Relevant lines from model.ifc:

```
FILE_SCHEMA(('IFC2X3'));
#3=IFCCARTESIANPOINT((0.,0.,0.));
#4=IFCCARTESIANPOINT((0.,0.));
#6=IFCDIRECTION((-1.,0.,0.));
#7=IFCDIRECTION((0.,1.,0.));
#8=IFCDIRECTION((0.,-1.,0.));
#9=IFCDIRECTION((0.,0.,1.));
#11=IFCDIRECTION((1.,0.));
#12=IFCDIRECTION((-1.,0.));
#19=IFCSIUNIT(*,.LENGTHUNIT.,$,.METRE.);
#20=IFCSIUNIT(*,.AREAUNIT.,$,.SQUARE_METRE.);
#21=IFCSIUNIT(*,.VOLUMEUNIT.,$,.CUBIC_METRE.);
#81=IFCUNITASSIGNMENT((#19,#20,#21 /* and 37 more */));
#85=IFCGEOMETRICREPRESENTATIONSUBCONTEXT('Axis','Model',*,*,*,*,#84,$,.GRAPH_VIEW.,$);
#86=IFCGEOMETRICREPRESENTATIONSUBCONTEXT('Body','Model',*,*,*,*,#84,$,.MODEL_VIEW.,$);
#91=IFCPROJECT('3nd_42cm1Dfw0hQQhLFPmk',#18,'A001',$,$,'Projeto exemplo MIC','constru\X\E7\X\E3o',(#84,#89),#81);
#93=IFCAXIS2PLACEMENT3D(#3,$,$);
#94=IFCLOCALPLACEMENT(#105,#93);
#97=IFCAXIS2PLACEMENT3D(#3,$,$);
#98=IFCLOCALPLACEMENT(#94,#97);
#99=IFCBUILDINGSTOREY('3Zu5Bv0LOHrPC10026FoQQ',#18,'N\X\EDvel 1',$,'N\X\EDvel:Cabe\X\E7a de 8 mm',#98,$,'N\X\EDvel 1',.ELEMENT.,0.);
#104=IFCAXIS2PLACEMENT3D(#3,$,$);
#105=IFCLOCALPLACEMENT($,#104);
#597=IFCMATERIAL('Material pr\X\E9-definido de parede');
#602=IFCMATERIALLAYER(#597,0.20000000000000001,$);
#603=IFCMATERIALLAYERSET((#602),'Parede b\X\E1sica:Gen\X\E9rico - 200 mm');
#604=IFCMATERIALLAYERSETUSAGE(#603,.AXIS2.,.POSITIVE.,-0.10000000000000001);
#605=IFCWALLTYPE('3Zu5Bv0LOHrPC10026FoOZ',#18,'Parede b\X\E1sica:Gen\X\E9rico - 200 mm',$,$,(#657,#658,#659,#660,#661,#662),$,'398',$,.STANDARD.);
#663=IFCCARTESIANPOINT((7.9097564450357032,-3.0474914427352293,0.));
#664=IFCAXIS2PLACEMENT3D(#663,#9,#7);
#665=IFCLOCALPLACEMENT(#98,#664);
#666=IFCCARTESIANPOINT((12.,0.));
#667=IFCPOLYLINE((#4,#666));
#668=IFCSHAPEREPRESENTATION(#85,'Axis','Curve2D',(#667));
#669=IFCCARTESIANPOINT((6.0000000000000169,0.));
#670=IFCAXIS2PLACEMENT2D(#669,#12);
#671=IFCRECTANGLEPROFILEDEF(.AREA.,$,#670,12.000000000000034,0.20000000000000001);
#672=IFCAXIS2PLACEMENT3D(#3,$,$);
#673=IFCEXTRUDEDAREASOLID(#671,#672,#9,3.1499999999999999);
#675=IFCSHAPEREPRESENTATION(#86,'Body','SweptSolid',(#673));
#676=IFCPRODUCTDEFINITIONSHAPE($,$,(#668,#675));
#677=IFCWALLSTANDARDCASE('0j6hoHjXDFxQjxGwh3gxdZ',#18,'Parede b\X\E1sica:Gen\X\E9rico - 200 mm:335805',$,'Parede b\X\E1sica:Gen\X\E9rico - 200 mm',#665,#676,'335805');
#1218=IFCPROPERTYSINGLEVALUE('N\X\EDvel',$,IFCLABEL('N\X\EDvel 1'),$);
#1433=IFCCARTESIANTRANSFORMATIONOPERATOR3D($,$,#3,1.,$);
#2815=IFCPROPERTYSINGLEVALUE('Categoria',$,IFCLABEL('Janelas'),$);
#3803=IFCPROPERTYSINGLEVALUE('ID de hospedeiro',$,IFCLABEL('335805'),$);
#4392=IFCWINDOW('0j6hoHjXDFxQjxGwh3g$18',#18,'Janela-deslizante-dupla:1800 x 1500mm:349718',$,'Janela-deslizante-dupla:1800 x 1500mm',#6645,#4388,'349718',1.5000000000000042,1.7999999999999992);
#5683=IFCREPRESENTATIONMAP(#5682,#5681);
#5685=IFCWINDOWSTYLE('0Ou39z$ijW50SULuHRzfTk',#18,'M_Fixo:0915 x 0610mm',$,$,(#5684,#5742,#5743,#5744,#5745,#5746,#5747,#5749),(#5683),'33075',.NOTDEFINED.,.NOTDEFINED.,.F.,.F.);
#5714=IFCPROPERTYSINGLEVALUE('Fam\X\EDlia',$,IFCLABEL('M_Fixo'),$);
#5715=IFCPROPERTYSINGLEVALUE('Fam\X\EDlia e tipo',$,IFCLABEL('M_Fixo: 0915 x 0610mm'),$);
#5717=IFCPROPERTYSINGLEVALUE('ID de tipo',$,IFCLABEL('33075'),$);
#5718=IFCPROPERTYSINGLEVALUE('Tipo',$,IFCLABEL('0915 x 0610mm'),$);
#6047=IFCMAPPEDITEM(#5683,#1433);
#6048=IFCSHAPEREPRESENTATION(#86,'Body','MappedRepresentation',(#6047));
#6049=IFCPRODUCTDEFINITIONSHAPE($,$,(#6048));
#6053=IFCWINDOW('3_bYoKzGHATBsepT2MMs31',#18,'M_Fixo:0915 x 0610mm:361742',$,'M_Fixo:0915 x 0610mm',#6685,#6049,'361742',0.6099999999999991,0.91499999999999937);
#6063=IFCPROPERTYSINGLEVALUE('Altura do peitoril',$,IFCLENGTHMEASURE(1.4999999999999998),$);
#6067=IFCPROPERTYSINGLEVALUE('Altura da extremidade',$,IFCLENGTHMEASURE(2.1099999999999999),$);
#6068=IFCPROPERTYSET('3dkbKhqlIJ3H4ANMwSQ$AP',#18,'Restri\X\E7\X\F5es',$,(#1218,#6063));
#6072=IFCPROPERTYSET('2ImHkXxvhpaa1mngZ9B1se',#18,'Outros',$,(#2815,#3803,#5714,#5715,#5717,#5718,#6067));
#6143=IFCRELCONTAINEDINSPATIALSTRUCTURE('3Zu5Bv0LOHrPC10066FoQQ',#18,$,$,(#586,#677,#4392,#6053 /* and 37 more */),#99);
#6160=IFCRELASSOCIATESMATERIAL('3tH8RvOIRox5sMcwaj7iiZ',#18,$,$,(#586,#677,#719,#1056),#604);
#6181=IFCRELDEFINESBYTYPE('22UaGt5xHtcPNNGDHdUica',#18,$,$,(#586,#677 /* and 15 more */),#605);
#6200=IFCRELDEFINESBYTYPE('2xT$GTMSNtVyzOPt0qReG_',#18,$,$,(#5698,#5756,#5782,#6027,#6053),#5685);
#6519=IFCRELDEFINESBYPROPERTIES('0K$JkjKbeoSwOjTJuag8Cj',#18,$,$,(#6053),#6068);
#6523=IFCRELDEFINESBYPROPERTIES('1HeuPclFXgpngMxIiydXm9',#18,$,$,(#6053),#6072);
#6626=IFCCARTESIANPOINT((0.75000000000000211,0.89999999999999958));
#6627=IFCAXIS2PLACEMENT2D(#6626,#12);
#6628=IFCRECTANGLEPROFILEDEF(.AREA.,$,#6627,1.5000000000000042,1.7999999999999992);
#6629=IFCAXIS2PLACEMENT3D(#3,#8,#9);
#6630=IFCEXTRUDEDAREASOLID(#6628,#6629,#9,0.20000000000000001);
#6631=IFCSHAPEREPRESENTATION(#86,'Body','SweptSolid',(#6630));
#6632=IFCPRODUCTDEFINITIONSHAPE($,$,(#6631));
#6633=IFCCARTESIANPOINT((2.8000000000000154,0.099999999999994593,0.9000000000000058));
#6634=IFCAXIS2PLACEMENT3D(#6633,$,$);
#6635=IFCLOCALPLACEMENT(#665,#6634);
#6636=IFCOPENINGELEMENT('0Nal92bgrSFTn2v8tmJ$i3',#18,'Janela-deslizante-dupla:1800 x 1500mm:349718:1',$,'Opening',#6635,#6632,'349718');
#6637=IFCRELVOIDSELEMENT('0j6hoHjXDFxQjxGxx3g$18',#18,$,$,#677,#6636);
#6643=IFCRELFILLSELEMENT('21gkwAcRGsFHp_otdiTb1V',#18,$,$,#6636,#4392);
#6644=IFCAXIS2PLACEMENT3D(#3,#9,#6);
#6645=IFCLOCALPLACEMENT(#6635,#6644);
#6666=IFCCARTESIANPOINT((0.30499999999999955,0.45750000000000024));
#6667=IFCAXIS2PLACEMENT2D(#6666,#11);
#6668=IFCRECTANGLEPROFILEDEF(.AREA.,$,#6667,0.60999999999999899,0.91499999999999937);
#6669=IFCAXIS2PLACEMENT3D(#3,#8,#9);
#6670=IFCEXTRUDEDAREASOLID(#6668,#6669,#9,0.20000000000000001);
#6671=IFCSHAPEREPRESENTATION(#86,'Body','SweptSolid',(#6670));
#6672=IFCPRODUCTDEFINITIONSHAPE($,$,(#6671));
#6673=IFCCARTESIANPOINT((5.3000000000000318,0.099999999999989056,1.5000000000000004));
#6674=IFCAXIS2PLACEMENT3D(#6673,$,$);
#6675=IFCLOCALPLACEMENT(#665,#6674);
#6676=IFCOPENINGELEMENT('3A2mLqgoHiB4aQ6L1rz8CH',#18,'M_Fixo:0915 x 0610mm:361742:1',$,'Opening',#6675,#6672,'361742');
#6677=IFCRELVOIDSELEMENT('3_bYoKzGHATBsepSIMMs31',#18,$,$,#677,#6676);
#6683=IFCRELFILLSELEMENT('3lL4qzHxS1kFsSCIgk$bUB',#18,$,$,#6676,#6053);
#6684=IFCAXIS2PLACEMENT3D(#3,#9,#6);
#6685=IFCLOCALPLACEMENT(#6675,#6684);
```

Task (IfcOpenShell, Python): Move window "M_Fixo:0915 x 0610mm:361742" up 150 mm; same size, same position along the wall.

```python
import numpy as np
import ifcopenshell
import ifcopenshell.api.geometry
import ifcopenshell.api.pset
import ifcopenshell.util.element
import ifcopenshell.util.placement
import ifcopenshell.util.unit

model = ifcopenshell.open("model.ifc")
unit_scale = ifcopenshell.util.unit.calculate_unit_scale(model)

window = model.by_guid("3_bYoKzGHATBsepT2MMs31")
opening = window.FillsVoids[0].RelatingOpeningElement
dz = 0.15

shift = np.array([0.0, 0.0, dz])
# The window is placed relative to its opening, so it follows when the opening moves.
matrix = ifcopenshell.util.placement.get_local_placement(opening.ObjectPlacement)
matrix[:3, 3] += shift
ifcopenshell.api.geometry.edit_object_placement(
    model, product=opening, matrix=matrix, is_si=False, should_transform_children=True
)

# Keep the stored heights in step.
pset = model.by_id(ifcopenshell.util.element.get_pset(window, "Restrições", should_inherit=False)["id"])
ifcopenshell.api.pset.edit_pset(model, pset=pset, properties={
    "Altura do peitoril": model.create_entity("IfcLengthMeasure", ifcopenshell.util.element.get_pset(window, "Restrições", "Altura do peitoril") + dz),
})
pset = model.by_id(ifcopenshell.util.element.get_pset(window, "Outros", should_inherit=False)["id"])
ifcopenshell.api.pset.edit_pset(model, pset=pset, properties={
    "Altura da extremidade": model.create_entity("IfcLengthMeasure", ifcopenshell.util.element.get_pset(window, "Outros", "Altura da extremidade") + dz),
})

print(f"moved by {dz * unit_scale:+.3f} m")

model.write("model_edited.ifc")
```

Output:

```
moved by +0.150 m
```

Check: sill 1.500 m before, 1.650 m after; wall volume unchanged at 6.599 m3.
